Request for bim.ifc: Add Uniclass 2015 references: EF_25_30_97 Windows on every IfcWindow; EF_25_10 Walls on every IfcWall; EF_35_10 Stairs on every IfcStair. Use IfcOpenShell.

First a look at what the model holds.

```python
import ifcopenshell

model = ifcopenshell.open("bim.ifc")
print(model.schema)
print("classifications:", [c.Name for c in model.by_type("IfcClassification")])
for ifc_class in ("IfcDoor", "IfcRoof", "IfcStair", "IfcWall", "IfcWindow"):
    print(ifc_class, len(model.by_type(ifc_class)))
```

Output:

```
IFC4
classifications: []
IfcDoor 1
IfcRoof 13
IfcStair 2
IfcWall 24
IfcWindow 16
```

```python
import ifcopenshell
import ifcopenshell.api.classification

model = ifcopenshell.open("bim.ifc")

system = ifcopenshell.api.classification.add_classification(model, classification="Uniclass 2015")

codes = {
    "IfcWindow": ("EF_25_30_97", "Windows"),
    "IfcWall": ("EF_25_10", "Walls"),
    "IfcStair": ("EF_35_10", "Stairs"),
}
for ifc_class, (code, name) in codes.items():
    products = model.by_type(ifc_class)
    ifcopenshell.api.classification.add_reference(
        model, products=products, classification=system, identification=code, name=name
    )
    print(code, len(products))

model.write("bim_updated.ifc")
```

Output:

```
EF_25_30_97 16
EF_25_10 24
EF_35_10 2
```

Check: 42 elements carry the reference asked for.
